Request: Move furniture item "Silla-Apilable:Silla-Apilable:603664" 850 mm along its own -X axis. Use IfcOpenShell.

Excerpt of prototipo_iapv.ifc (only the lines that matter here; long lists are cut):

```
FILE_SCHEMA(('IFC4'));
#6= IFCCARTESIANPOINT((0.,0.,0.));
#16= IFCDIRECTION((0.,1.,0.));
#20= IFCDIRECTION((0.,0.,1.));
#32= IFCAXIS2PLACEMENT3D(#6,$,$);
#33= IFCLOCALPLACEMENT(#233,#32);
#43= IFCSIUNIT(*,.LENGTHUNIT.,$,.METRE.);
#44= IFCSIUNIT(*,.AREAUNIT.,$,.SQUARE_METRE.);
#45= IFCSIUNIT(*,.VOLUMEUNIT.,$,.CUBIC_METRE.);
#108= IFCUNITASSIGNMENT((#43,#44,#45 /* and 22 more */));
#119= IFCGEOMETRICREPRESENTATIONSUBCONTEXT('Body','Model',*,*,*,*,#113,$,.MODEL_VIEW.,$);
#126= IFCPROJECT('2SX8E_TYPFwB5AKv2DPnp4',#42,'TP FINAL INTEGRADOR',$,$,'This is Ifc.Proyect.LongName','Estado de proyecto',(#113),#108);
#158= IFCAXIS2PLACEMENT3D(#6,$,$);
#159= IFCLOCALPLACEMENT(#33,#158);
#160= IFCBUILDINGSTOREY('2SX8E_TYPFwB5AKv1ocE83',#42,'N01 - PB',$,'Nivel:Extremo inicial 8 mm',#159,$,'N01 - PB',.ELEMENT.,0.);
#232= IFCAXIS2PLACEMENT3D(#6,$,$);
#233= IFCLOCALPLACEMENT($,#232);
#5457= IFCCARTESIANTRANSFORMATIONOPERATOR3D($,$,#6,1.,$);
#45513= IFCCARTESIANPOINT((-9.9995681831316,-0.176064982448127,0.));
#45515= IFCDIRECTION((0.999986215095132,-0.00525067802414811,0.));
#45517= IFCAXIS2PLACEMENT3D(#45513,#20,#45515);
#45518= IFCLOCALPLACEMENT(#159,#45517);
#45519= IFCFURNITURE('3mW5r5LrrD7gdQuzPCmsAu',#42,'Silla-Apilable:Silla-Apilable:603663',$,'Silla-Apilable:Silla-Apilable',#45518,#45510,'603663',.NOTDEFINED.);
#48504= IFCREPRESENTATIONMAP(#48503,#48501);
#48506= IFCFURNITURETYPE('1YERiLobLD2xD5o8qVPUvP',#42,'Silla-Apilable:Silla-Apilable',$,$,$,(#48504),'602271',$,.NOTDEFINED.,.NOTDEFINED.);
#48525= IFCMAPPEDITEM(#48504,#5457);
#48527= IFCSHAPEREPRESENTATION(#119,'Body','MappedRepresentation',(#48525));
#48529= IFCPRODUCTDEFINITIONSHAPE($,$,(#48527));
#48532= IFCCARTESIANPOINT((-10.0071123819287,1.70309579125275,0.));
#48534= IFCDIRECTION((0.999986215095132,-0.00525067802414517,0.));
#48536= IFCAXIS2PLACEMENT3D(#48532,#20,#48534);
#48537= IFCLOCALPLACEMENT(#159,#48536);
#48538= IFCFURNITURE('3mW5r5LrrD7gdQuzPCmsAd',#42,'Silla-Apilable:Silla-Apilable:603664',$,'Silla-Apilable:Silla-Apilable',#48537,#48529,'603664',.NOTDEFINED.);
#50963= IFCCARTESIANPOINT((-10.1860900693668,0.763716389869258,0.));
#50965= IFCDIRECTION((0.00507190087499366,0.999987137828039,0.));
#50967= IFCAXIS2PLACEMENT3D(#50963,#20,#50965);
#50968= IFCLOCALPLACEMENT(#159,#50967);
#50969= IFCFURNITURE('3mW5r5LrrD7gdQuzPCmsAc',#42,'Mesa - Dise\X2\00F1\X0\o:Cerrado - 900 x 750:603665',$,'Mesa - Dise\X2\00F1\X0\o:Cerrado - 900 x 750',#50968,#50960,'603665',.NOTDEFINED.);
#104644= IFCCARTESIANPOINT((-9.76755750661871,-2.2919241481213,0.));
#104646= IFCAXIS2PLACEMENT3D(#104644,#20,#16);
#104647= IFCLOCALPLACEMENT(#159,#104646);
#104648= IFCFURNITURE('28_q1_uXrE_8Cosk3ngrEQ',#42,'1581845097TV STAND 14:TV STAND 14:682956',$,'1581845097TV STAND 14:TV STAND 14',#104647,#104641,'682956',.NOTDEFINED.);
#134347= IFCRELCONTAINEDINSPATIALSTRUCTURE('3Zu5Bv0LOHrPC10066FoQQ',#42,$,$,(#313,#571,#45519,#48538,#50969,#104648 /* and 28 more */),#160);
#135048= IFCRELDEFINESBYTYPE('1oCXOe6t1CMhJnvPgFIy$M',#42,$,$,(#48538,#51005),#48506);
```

```python
import ifcopenshell
import ifcopenshell.api.geometry
import ifcopenshell.util.placement

model = ifcopenshell.open("prototipo_iapv.ifc")

item = model.by_guid("3mW5r5LrrD7gdQuzPCmsAd")
matrix = ifcopenshell.util.placement.get_local_placement(item.ObjectPlacement)
matrix[:3, 3] -= matrix[:3, 0] * 0.85
ifcopenshell.api.geometry.edit_object_placement(model, product=item, matrix=matrix, is_si=False)

print(ifcopenshell.util.placement.get_local_placement(item.ObjectPlacement).round(3) + 0.0)

model.write("prototipo_iapv_updated.ifc")
```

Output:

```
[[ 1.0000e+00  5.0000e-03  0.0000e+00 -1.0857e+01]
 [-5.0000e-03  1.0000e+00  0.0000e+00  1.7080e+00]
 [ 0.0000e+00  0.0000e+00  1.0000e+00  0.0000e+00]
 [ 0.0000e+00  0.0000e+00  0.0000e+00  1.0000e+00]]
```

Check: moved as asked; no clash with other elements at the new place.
